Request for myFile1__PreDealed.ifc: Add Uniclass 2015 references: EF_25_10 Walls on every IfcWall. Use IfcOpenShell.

First a look at what the model holds.

```python
import ifcopenshell

model = ifcopenshell.open("myFile1__PreDealed.ifc")
print(model.schema)
print("classifications:", [c.Name for c in model.by_type("IfcClassification")])
for ifc_class in ("IfcDoor", "IfcRoof", "IfcStair", "IfcWall", "IfcWindow"):
    print(ifc_class, len(model.by_type(ifc_class)))
```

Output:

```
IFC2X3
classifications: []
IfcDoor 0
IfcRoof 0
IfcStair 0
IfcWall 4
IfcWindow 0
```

```python
import ifcopenshell
import ifcopenshell.api.classification

model = ifcopenshell.open("myFile1__PreDealed.ifc")

# IFC2X3 requires Source and Edition and has no link from the project to the system.
system = model.create_entity("IfcClassification", Source="NBS", Edition="2015", Name="Uniclass 2015")

codes = {
    "IfcWall": ("EF_25_10", "Walls"),
}
for ifc_class, (code, name) in codes.items():
    products = model.by_type(ifc_class)
    ifcopenshell.api.classification.add_reference(
        model, products=products, classification=system, identification=code, name=name
    )
    print(code, len(products))

model.write("myFile1__PreDealed_rev.ifc")
```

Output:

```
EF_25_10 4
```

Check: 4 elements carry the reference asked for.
